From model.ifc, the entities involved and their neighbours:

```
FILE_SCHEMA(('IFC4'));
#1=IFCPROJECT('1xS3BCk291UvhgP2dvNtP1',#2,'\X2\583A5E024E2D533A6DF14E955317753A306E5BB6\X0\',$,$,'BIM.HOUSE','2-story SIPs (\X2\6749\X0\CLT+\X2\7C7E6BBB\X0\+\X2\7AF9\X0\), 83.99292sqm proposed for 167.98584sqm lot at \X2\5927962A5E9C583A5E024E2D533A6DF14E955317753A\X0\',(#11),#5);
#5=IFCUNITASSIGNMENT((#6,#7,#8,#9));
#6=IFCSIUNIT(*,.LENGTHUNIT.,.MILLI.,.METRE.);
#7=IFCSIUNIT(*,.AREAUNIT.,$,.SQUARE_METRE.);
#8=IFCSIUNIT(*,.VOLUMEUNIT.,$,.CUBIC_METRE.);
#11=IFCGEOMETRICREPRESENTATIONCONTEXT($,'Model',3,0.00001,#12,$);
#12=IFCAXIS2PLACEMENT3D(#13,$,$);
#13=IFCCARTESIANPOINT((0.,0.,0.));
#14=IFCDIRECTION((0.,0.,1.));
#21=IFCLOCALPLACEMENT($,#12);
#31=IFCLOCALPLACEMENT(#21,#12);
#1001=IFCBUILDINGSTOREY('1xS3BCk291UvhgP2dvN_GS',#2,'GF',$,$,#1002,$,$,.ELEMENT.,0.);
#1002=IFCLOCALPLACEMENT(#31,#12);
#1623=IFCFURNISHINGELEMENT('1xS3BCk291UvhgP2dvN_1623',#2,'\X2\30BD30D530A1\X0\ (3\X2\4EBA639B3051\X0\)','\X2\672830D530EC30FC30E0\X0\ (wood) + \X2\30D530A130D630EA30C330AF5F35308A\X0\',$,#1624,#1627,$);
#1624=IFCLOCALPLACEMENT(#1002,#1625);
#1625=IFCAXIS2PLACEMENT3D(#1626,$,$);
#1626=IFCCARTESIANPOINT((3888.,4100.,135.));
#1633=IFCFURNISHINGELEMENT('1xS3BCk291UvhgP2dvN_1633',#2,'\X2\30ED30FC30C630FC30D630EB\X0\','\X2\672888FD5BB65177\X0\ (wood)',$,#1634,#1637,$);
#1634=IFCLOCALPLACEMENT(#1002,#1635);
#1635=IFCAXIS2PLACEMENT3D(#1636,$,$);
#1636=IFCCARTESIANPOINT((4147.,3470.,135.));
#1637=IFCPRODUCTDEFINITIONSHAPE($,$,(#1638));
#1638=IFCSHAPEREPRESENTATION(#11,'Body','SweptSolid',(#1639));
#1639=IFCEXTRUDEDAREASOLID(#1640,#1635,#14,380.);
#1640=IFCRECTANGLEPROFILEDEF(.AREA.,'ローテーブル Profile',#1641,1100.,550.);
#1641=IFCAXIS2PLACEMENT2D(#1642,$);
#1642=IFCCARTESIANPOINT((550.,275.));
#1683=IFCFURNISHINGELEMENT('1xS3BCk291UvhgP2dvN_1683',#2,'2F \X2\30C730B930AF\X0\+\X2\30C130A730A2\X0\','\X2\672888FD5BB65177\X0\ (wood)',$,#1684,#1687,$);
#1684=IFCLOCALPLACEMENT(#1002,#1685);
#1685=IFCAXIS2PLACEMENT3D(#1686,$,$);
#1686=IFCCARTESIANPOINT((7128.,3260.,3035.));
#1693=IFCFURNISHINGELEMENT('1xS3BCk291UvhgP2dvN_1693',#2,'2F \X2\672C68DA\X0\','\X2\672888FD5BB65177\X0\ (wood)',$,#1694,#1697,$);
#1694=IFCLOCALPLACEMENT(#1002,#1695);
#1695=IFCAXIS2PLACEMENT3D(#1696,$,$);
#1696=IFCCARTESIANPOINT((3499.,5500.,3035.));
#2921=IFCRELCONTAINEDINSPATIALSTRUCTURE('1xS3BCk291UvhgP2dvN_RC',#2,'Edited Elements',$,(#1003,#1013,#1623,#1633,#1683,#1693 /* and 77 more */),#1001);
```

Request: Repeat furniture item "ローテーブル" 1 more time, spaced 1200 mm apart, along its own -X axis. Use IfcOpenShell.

```python
import ifcopenshell
import ifcopenshell.api.geometry
import ifcopenshell.api.root
import ifcopenshell.util.element
import ifcopenshell.util.placement
import ifcopenshell.util.unit

model = ifcopenshell.open("model.ifc")
unit_scale = ifcopenshell.util.unit.calculate_unit_scale(model)


def reuse_history(source, copy):
    """copy_class also copies each property set's owner history, people and application; keep the originals."""
    for rel in copy.IsDefinedBy:
        if rel.is_a("IfcRelDefinesByProperties") and (history := rel.RelatingPropertyDefinition.OwnerHistory):
            rel.RelatingPropertyDefinition.OwnerHistory = source.OwnerHistory
            ifcopenshell.util.element.remove_deep2(model, history)


source = model.by_guid("1xS3BCk291UvhgP2dvN_1633")
base = ifcopenshell.util.placement.get_local_placement(source.ObjectPlacement)
step = -base[:3, 0] * 1.2 / unit_scale

for i in range(1, 2):
    copy = ifcopenshell.api.root.copy_class(model, product=source)
    copy.Representation = ifcopenshell.util.element.copy_deep(
        model, source.Representation, exclude=["IfcGeometricRepresentationContext", "IfcRepresentationMap"]
    )
    reuse_history(source, copy)
    matrix = base.copy()
    matrix[:3, 3] += i * step
    print("added at", matrix[:3, 3].round(3) + 0.0)
    ifcopenshell.api.geometry.edit_object_placement(model, product=copy, matrix=matrix, is_si=False)

model.write("model_rev.ifc")
```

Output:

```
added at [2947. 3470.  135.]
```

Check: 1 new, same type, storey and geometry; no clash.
